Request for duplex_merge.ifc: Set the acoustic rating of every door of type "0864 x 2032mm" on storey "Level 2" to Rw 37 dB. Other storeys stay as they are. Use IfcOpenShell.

First a look at what the model holds.

```python
import ifcopenshell
import ifcopenshell.util.element

model = ifcopenshell.open("duplex_merge.ifc")
print(model.schema)
storey = next(s for s in model.by_type("IfcBuildingStorey") if s.Name == "Level 2")
doors = [e for e in ifcopenshell.util.element.get_decomposition(storey) if e.is_a("IfcDoor")]
seen = {}
for e in doors:
    element_type = ifcopenshell.util.element.get_type(e)
    key = (element_type.Name if element_type != e and element_type else None, ifcopenshell.util.element.get_pset(e, "Pset_DoorCommon", "AcousticRating"))
    seen[key] = seen.get(key, 0) + 1
for (name, value), count in sorted(seen.items(), key=str):
    print(count, "x", name, "|", value)
```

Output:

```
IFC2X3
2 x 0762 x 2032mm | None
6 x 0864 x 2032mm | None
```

```python
import ifcopenshell
import ifcopenshell.api.pset
import ifcopenshell.util.element

model = ifcopenshell.open("duplex_merge.ifc")

storey = next(s for s in model.by_type("IfcBuildingStorey") if s.Name == "Level 2")
doors = [e for e in ifcopenshell.util.element.get_decomposition(storey) if e.is_a("IfcDoor")]

count = 0
for e in doors:
    element_type = ifcopenshell.util.element.get_type(e)
    if element_type in (None, e) or element_type.Name != "0864 x 2032mm":
        continue
    # add_pset returns the element's existing set when there is one.
    pset = ifcopenshell.api.pset.add_pset(model, product=e, name="Pset_DoorCommon")
    ifcopenshell.api.pset.edit_pset(model, pset=pset, properties={"AcousticRating": "Rw 37 dB"})
    count += 1

print(count, "doors updated")

model.write("duplex_merge_v2.ifc")
```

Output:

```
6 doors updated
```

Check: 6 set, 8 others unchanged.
